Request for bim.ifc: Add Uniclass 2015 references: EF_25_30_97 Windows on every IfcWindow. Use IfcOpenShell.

First a look at what the model holds.

```python
import ifcopenshell

model = ifcopenshell.open("bim.ifc")
print(model.schema)
print("classifications:", [c.Name for c in model.by_type("IfcClassification")])
for ifc_class in ("IfcDoor", "IfcRoof", "IfcStair", "IfcWall", "IfcWindow"):
    print(ifc_class, len(model.by_type(ifc_class)))
```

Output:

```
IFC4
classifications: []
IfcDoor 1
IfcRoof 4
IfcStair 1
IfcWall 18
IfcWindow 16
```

```python
import ifcopenshell
import ifcopenshell.api.classification

model = ifcopenshell.open("bim.ifc")

system = ifcopenshell.api.classification.add_classification(model, classification="Uniclass 2015")

codes = {
    "IfcWindow": ("EF_25_30_97", "Windows"),
}
for ifc_class, (code, name) in codes.items():
    products = model.by_type(ifc_class)
    ifcopenshell.api.classification.add_reference(
        model, products=products, classification=system, identification=code, name=name
    )
    print(code, len(products))

model.write("bim_updated.ifc")
```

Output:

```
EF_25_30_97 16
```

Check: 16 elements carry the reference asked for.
